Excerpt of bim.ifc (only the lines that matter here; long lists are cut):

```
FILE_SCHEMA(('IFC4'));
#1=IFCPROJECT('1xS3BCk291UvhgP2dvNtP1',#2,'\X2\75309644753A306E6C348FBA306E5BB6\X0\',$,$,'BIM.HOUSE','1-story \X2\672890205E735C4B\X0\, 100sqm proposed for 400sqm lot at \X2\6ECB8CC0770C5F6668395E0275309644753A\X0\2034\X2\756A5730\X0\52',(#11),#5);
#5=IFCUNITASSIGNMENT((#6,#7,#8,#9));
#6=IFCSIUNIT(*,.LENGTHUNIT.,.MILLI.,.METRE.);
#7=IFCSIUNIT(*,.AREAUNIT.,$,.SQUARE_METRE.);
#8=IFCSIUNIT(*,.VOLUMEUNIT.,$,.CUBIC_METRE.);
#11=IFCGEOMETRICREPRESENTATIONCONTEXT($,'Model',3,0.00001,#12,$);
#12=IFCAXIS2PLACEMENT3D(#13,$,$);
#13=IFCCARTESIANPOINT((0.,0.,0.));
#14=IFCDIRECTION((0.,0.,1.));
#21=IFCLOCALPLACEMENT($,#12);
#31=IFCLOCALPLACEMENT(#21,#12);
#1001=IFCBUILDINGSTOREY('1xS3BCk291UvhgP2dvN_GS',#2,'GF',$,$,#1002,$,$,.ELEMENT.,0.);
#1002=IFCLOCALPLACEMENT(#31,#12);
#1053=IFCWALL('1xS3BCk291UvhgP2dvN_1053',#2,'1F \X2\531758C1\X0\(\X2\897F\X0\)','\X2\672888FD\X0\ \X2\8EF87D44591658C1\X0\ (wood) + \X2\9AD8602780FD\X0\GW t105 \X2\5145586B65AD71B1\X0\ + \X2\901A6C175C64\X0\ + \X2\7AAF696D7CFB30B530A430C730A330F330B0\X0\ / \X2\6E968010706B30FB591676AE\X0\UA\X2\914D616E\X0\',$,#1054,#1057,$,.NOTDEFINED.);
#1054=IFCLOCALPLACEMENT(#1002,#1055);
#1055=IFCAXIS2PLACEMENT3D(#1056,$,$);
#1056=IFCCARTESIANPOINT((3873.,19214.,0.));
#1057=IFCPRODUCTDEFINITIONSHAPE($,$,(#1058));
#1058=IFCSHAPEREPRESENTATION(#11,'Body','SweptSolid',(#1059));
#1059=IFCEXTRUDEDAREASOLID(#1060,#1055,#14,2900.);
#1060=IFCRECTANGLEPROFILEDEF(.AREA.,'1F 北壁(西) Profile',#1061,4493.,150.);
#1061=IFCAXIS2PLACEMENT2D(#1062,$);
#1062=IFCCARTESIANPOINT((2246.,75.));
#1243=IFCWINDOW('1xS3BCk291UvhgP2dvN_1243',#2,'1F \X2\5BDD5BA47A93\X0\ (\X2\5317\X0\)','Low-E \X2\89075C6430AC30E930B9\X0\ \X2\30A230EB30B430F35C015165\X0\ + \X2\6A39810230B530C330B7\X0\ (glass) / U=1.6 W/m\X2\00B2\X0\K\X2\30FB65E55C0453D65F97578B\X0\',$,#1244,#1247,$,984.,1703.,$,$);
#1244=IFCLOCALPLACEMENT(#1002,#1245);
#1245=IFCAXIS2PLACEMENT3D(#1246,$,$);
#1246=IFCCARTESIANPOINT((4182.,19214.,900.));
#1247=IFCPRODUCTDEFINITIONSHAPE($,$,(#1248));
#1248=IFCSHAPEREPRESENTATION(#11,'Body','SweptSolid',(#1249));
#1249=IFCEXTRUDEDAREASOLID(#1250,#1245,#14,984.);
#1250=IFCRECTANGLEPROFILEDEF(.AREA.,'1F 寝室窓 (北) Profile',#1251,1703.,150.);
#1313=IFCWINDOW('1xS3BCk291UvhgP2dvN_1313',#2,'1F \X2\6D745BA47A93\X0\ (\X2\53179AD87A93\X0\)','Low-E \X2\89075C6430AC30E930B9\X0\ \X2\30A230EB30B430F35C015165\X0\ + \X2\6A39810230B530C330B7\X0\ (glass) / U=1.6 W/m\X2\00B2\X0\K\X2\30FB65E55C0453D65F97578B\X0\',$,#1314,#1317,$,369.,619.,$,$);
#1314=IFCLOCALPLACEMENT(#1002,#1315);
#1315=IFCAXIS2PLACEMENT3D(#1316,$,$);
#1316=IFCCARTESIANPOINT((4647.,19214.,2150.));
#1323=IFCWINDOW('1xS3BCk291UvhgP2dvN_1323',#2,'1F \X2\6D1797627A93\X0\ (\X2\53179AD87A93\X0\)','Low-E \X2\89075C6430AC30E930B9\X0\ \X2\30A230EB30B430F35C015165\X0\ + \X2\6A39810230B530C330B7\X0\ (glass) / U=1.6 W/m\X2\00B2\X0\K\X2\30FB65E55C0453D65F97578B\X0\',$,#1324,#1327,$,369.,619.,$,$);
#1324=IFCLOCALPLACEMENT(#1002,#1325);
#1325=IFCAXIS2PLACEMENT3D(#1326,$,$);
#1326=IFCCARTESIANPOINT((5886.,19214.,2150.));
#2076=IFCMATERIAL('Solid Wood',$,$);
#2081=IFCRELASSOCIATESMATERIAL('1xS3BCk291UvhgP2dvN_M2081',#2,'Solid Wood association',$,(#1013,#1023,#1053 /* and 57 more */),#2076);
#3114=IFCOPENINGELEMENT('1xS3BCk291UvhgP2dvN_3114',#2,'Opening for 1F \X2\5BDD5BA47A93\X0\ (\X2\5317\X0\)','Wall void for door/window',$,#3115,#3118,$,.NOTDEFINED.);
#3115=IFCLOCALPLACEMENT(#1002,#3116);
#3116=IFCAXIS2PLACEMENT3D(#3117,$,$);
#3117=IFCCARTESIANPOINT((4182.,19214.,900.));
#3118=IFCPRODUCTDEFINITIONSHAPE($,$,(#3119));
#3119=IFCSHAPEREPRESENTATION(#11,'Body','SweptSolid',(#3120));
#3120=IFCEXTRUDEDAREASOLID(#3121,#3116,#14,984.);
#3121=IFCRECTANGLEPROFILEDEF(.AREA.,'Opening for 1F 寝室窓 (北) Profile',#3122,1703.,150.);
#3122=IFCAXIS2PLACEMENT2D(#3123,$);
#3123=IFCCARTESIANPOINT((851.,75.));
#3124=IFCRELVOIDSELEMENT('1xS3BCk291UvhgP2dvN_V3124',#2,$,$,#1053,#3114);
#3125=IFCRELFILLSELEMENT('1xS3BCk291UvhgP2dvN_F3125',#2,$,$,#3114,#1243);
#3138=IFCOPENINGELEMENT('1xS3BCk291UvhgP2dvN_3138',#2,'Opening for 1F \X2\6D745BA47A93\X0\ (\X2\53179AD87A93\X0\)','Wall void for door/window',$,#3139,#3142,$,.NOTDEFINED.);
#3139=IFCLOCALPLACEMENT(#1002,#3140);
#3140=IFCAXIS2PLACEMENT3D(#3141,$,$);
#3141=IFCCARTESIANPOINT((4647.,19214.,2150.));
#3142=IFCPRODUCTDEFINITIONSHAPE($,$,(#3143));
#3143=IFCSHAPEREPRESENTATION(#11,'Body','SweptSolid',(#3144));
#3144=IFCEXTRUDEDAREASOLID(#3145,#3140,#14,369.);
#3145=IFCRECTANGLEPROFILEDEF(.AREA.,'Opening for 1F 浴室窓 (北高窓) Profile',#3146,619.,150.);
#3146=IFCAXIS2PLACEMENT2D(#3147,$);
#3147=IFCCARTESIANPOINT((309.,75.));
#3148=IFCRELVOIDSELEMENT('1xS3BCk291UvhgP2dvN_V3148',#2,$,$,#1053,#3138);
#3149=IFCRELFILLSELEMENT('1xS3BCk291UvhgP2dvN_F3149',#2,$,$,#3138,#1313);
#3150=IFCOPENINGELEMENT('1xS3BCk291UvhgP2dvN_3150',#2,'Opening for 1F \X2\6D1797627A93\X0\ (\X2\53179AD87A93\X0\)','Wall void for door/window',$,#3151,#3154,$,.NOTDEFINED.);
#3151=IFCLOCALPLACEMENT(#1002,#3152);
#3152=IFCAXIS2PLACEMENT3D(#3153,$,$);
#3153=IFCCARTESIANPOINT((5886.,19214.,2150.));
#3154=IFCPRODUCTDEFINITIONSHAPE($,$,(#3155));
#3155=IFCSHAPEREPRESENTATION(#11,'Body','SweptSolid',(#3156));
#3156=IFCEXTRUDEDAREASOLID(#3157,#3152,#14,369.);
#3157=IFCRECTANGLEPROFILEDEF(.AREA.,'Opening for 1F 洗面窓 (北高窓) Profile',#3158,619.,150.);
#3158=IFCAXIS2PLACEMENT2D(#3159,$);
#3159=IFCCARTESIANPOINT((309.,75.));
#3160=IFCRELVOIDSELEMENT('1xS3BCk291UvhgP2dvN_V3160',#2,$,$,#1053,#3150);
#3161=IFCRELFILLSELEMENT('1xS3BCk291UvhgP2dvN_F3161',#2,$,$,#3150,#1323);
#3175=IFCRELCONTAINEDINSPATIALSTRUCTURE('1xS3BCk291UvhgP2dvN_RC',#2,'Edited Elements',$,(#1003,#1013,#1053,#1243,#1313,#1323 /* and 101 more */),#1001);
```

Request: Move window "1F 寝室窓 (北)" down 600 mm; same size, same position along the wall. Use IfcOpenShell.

```python
import numpy as np
import ifcopenshell
import ifcopenshell.api.geometry
import ifcopenshell.util.placement
import ifcopenshell.util.unit

model = ifcopenshell.open("bim.ifc")
unit_scale = ifcopenshell.util.unit.calculate_unit_scale(model)

window = model.by_guid("1xS3BCk291UvhgP2dvN_1243")
opening = window.FillsVoids[0].RelatingOpeningElement
dz = -0.6 / unit_scale

shift = np.array([0.0, 0.0, dz])
# The window is not placed relative to its opening, so move both.
for product in (opening, window):
    matrix = ifcopenshell.util.placement.get_local_placement(product.ObjectPlacement)
    matrix[:3, 3] += shift
    ifcopenshell.api.geometry.edit_object_placement(model, product=product, matrix=matrix, is_si=False)

print(f"moved by {dz * unit_scale:+.3f} m")

model.write("bim_edited.ifc")
```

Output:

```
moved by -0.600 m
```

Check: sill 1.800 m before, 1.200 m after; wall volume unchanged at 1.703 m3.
